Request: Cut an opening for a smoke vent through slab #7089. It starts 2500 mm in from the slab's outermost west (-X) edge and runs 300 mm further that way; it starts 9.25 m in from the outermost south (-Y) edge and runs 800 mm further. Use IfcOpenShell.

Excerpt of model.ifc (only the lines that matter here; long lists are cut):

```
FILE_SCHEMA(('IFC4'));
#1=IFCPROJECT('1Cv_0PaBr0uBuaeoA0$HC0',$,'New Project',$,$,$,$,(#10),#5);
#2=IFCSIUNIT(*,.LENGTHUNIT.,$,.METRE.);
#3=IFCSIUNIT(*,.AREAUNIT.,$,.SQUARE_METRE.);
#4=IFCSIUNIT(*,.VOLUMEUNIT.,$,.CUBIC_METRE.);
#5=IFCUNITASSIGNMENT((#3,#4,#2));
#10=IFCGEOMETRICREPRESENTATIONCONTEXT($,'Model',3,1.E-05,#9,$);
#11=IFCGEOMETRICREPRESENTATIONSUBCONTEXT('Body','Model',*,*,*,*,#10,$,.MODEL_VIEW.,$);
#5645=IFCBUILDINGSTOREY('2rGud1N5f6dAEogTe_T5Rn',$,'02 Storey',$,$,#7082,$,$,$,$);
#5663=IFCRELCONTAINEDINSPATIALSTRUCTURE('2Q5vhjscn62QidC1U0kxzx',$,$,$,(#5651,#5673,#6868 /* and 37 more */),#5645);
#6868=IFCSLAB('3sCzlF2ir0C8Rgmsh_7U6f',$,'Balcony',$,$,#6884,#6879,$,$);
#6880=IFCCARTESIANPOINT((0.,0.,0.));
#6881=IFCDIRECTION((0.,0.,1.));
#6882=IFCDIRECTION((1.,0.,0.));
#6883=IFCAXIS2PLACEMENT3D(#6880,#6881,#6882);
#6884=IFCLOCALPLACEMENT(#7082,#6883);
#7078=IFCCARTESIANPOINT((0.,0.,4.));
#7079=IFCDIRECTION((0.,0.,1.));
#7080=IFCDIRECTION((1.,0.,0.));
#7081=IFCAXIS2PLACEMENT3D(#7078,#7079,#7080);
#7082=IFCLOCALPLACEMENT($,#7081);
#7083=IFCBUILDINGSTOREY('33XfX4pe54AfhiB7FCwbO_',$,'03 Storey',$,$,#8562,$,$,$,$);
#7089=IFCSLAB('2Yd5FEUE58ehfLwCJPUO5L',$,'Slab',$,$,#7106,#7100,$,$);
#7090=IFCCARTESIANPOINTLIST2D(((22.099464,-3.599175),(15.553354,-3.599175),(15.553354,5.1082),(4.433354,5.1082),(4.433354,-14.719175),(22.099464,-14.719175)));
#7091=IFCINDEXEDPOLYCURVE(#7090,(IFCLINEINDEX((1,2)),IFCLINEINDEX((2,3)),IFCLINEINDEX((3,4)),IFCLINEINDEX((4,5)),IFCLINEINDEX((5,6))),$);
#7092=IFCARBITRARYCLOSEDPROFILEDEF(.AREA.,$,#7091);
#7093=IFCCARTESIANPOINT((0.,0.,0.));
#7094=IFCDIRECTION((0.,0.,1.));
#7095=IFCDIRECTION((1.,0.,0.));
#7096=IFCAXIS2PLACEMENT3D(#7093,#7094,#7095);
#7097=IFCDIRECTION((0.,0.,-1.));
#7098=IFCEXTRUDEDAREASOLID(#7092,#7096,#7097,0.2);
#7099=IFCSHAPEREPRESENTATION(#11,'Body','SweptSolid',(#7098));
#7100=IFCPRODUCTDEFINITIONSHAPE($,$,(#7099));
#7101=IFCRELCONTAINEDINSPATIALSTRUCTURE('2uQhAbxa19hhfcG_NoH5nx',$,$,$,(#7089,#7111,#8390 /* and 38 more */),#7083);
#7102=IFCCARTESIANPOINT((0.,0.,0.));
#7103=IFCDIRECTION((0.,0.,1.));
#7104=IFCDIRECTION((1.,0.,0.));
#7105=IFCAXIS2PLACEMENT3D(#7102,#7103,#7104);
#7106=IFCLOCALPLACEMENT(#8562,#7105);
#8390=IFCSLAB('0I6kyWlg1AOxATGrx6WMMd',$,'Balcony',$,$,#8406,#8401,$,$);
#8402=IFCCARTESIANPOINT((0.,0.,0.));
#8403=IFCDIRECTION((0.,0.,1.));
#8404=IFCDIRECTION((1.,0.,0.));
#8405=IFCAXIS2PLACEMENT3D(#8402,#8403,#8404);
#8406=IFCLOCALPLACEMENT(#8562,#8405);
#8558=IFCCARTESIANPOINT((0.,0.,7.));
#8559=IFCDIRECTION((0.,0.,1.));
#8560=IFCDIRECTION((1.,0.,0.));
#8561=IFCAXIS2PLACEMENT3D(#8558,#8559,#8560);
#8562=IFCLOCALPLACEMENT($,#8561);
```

```python
import numpy as np
import ifcopenshell
import ifcopenshell.api.feature
import ifcopenshell.api.geometry
import ifcopenshell.api.root
import ifcopenshell.geom
import ifcopenshell.util.placement
import ifcopenshell.util.representation
import ifcopenshell.util.shape
import ifcopenshell.util.unit

model = ifcopenshell.open("model.ifc")
unit_scale = ifcopenshell.util.unit.calculate_unit_scale(model)
settings = ifcopenshell.geom.settings()


def volume(element):
    """Net volume in cubic metres, openings subtracted."""
    shape = ifcopenshell.geom.create_shape(settings, element)
    return ifcopenshell.util.shape.get_volume(shape.geometry)


slab = model.by_guid("2Yd5FEUE58ehfLwCJPUO5L")
before = volume(slab)

# Extent in the slab's own axes, in metres. The edges named are its -X and -Y sides.
slab_shape = ifcopenshell.geom.create_shape(settings, slab)
vertices = ifcopenshell.util.shape.get_vertices(slab_shape.geometry)
x_min, y_min, bottom = vertices.min(axis=0)
top = vertices[:, 2].max()

opening = ifcopenshell.api.root.create_entity(model, ifc_class="IfcOpeningElement", name="Smoke vent opening", predefined_type="OPENING")
context = ifcopenshell.util.representation.get_context(model, "Model", "Body", "MODEL_VIEW")
width, depth = 0.3, 0.8
outline = [(0.0, 0.0), (width, 0.0), (width, depth), (0.0, depth), (0.0, 0.0)]
# Overshoot both faces by 50 mm so the cut is clean.
shape = ifcopenshell.api.geometry.add_slab_representation(
    model, context=context, depth=top - bottom + 0.1, polyline=outline
)
ifcopenshell.api.geometry.assign_representation(model, product=opening, representation=shape)

matrix = ifcopenshell.util.placement.get_local_placement(slab.ObjectPlacement)
matrix[:, 3] = matrix @ np.append(np.array([x_min + 2.5, y_min + 9.25, bottom - 0.05]) / unit_scale, 1.0)
ifcopenshell.api.geometry.edit_object_placement(model, product=opening, matrix=matrix, is_si=False)
ifcopenshell.api.feature.add_feature(model, feature=opening, element=slab)

after = volume(slab)

print(f"slab volume {before:.3f} -> {after:.3f} m3")

model.write("model_edited.ifc")
```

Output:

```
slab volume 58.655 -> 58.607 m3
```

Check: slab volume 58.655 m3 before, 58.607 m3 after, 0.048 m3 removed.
